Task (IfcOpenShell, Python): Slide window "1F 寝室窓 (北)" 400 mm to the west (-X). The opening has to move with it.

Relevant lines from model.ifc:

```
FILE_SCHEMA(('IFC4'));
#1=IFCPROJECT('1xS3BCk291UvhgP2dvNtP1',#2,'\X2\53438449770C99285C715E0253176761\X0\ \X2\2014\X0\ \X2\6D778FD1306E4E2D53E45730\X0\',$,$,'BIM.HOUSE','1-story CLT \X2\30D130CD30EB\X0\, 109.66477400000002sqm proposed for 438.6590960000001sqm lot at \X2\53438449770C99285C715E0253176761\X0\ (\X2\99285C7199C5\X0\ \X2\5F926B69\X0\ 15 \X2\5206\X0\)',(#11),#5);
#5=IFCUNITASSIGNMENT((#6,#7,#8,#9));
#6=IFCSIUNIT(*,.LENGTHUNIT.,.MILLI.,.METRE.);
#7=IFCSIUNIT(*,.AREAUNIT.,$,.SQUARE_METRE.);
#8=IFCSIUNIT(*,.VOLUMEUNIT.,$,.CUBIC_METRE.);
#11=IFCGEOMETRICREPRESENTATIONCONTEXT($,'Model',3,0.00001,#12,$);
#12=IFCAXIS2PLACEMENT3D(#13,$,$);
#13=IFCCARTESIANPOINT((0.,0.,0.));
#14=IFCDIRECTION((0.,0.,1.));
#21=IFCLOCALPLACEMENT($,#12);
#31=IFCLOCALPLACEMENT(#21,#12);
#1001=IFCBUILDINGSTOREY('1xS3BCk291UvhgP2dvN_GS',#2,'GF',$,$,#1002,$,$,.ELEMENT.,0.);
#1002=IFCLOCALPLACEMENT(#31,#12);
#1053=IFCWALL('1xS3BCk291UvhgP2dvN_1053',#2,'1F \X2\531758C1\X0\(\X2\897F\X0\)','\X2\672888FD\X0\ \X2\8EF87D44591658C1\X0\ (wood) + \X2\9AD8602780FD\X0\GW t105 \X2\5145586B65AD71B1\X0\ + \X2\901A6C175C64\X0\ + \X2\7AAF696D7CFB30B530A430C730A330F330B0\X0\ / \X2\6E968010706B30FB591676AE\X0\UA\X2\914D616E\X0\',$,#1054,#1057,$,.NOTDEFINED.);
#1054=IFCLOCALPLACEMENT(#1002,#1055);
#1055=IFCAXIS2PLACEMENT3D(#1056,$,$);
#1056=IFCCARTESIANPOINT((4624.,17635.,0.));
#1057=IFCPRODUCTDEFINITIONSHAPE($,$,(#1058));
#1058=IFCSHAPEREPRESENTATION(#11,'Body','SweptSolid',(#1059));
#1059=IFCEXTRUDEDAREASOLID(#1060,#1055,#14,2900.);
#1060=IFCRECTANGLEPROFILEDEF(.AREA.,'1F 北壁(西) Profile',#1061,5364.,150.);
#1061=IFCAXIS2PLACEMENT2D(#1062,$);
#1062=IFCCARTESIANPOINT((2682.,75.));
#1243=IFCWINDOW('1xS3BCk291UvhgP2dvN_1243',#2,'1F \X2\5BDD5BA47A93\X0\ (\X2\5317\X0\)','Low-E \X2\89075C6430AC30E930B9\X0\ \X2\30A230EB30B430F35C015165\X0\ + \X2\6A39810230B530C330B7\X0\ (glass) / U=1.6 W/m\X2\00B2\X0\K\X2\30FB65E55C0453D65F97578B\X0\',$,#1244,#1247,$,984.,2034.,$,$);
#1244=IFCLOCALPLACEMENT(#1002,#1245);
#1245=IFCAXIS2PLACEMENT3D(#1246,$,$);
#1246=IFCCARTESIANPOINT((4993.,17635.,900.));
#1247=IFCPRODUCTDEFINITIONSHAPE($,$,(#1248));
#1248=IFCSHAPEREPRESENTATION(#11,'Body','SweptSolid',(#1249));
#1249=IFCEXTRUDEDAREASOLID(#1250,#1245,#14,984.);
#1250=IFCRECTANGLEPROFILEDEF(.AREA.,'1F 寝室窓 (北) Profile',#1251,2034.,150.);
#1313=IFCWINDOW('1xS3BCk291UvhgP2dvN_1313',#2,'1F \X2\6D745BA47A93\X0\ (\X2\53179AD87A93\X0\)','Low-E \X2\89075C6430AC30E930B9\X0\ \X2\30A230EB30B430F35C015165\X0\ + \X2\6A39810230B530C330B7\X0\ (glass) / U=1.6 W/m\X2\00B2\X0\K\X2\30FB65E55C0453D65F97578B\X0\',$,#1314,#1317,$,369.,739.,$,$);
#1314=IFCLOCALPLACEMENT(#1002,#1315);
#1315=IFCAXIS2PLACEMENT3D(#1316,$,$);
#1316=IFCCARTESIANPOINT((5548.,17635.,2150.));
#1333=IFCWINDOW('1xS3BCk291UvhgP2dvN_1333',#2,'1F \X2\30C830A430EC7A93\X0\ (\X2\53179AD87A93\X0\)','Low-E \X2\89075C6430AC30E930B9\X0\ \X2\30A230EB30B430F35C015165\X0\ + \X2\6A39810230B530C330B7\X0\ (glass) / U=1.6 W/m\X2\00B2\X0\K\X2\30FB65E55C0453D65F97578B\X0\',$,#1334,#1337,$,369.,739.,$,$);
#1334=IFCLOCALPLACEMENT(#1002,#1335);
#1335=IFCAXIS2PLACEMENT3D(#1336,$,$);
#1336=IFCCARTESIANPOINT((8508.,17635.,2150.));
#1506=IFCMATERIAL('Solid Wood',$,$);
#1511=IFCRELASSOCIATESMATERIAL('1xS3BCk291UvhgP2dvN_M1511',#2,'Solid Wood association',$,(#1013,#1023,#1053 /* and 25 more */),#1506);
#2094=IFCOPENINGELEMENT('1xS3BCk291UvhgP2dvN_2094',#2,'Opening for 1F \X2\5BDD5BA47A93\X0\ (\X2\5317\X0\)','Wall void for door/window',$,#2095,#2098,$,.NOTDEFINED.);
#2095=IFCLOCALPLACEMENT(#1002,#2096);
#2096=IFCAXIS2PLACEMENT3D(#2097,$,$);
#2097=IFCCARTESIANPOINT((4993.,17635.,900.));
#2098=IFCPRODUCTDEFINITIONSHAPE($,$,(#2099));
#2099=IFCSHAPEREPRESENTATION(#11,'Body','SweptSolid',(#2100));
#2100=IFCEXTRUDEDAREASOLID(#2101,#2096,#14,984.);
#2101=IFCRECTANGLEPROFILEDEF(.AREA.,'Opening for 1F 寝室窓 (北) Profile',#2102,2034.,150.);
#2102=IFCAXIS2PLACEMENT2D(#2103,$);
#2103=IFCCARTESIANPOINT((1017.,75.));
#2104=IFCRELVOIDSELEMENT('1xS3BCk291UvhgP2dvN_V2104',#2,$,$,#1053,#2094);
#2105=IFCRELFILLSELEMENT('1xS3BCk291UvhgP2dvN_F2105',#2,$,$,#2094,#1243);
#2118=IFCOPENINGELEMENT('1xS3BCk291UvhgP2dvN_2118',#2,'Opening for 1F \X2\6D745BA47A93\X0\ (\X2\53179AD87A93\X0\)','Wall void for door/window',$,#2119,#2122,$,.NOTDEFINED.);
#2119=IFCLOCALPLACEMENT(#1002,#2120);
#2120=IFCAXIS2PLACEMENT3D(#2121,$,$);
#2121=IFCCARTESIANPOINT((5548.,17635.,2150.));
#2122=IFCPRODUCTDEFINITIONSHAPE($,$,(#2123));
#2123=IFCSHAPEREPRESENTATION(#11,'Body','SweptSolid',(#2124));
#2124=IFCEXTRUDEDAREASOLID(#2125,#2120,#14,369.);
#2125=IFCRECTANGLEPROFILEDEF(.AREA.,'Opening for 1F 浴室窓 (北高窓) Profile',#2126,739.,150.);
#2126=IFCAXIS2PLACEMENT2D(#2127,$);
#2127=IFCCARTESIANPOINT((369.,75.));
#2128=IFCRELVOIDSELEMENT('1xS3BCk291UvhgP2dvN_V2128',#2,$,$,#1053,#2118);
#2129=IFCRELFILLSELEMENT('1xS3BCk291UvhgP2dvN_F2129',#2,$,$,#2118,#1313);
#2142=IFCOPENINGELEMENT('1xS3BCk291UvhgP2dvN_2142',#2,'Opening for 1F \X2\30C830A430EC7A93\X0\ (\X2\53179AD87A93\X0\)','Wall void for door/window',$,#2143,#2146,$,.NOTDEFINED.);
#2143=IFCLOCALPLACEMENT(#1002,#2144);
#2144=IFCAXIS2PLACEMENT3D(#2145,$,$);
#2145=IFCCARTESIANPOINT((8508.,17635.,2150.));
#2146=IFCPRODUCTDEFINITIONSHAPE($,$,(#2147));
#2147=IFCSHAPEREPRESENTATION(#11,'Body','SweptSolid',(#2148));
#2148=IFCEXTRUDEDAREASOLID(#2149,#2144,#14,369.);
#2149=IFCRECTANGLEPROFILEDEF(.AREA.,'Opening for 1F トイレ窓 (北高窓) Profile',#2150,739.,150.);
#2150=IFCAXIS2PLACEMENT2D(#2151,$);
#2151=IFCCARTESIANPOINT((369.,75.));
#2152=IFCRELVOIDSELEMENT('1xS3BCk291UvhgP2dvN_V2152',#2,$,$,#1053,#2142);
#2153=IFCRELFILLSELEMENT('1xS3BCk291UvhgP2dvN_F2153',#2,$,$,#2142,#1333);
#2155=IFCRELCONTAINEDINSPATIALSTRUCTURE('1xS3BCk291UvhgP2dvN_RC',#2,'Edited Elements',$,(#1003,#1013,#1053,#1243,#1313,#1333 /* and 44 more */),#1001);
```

```python
import ifcopenshell
import ifcopenshell.api.geometry
import ifcopenshell.util.placement

model = ifcopenshell.open("model.ifc")

window = model.by_guid("1xS3BCk291UvhgP2dvN_1243")
opening = window.FillsVoids[0].RelatingOpeningElement
wall = opening.VoidsElements[0].RelatingBuildingElement

wall_matrix = ifcopenshell.util.placement.get_local_placement(wall.ObjectPlacement)
shift = wall_matrix[:3, 0] * -400.0
before = ifcopenshell.util.placement.get_local_placement(window.ObjectPlacement)[:3, 3].copy()

# The window is not placed relative to its opening, so move both.
for product in (opening, window):
    matrix = ifcopenshell.util.placement.get_local_placement(product.ObjectPlacement)
    matrix[:3, 3] += shift
    ifcopenshell.api.geometry.edit_object_placement(model, product=product, matrix=matrix, is_si=False)

after = ifcopenshell.util.placement.get_local_placement(window.ObjectPlacement)[:3, 3]
print("window moved by", (after - before).round(3) + 0.0)

model.write("model-out.ifc")
```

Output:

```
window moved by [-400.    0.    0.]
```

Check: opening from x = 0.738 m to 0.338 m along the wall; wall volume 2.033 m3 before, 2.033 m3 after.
